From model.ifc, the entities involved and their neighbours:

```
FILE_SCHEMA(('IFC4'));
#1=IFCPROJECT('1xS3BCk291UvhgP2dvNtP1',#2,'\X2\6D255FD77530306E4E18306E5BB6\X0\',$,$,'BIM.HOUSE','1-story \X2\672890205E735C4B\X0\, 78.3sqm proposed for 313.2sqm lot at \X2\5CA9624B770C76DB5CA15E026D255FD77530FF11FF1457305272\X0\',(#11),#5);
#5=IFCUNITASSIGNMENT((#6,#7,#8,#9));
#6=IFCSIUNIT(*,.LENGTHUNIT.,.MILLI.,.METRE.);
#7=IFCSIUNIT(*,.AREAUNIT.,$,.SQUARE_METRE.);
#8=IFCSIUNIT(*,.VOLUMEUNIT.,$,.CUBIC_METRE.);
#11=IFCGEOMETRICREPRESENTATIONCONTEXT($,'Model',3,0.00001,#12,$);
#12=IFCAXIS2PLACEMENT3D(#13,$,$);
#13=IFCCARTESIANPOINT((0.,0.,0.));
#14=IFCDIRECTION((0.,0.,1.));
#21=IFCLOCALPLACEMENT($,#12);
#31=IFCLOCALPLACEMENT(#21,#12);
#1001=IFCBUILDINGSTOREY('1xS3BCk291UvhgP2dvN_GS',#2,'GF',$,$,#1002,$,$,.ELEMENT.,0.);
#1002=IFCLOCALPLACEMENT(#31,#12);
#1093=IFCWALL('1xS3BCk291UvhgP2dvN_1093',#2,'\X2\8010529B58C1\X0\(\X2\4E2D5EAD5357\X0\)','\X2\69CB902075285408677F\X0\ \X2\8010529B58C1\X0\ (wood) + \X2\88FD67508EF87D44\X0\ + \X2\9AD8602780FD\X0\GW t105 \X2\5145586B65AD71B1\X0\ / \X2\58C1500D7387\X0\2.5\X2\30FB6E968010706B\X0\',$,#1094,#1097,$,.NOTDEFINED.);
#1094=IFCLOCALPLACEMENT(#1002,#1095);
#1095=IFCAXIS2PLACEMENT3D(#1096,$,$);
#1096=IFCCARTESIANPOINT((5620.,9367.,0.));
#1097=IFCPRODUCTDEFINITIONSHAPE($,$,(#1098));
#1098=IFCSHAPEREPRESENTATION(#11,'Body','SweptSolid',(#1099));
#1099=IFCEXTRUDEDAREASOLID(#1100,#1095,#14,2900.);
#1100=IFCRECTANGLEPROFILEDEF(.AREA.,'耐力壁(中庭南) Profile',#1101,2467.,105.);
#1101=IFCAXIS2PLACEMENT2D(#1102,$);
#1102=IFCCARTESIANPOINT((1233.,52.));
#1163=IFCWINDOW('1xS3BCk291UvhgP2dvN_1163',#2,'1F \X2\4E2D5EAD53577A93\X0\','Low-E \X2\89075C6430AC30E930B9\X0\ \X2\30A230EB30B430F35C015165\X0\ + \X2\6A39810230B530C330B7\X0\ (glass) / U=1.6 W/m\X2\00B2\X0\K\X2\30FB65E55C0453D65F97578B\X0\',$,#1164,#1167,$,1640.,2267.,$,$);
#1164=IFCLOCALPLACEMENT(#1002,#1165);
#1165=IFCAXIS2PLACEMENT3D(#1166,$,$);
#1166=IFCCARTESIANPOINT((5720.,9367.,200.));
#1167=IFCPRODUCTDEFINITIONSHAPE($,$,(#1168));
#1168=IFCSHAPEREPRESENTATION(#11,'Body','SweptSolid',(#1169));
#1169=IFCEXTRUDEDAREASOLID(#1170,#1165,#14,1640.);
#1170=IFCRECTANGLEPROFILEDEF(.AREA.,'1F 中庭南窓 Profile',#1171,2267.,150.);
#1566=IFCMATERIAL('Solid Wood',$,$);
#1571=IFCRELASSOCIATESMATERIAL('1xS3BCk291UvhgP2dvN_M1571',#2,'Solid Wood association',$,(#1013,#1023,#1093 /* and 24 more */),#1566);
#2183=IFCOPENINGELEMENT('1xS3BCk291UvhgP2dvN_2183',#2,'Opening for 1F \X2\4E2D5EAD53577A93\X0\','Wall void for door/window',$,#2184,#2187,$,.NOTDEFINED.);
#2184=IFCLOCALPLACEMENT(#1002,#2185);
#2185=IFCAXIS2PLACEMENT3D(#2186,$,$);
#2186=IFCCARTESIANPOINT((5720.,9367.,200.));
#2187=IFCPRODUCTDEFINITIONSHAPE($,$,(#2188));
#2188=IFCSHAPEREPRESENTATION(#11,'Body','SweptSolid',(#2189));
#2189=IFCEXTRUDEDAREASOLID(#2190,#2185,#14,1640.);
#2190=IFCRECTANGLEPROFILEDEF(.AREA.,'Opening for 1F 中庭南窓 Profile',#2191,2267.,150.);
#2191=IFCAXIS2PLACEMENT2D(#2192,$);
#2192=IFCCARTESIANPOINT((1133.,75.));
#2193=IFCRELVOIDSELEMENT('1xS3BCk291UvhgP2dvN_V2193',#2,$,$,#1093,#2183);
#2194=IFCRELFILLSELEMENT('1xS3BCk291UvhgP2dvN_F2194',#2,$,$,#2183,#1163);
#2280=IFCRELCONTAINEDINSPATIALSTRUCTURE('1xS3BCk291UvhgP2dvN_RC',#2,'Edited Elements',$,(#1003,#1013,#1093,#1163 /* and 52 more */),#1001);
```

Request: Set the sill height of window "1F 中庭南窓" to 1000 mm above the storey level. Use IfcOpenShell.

```python
import numpy as np
import ifcopenshell
import ifcopenshell.api.geometry
import ifcopenshell.geom
import ifcopenshell.util.element
import ifcopenshell.util.placement
import ifcopenshell.util.shape
import ifcopenshell.util.unit

model = ifcopenshell.open("model.ifc")
unit_scale = ifcopenshell.util.unit.calculate_unit_scale(model)

window = model.by_id(1163)
opening = window.FillsVoids[0].RelatingOpeningElement
storey = ifcopenshell.util.element.get_container(window, ifc_class="IfcBuildingStorey")
level = ifcopenshell.util.placement.get_local_placement(storey.ObjectPlacement)[2, 3]

# The opening's origin need not be at the sill, so measure its lowest point.
shape = ifcopenshell.geom.create_shape(ifcopenshell.geom.settings(), opening)
bottom = ifcopenshell.util.shape.get_shape_bottom_elevation(shape, shape.geometry) / unit_scale
dz = level + 1 / unit_scale - bottom

shift = np.array([0.0, 0.0, dz])
# The window is not placed relative to its opening, so move both.
for product in (opening, window):
    matrix = ifcopenshell.util.placement.get_local_placement(product.ObjectPlacement)
    matrix[:3, 3] += shift
    ifcopenshell.api.geometry.edit_object_placement(model, product=product, matrix=matrix, is_si=False)

print(f"moved by {dz * unit_scale:+.3f} m")

model.write("model_edited.ifc")
```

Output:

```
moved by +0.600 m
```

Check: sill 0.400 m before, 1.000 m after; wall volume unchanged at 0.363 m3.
